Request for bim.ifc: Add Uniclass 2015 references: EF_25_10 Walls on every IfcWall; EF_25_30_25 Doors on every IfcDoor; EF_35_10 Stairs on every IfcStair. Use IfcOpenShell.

First a look at what the model holds.

```python
import ifcopenshell

model = ifcopenshell.open("bim.ifc")
print(model.schema)
print("classifications:", [c.Name for c in model.by_type("IfcClassification")])
for ifc_class in ("IfcDoor", "IfcRoof", "IfcStair", "IfcWall", "IfcWindow"):
    print(ifc_class, len(model.by_type(ifc_class)))
```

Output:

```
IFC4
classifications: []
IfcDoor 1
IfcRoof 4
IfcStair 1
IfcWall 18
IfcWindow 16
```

```python
import ifcopenshell
import ifcopenshell.api.classification

model = ifcopenshell.open("bim.ifc")

system = ifcopenshell.api.classification.add_classification(model, classification="Uniclass 2015")

codes = {
    "IfcWall": ("EF_25_10", "Walls"),
    "IfcDoor": ("EF_25_30_25", "Doors"),
    "IfcStair": ("EF_35_10", "Stairs"),
}
for ifc_class, (code, name) in codes.items():
    products = model.by_type(ifc_class)
    ifcopenshell.api.classification.add_reference(
        model, products=products, classification=system, identification=code, name=name
    )
    print(code, len(products))

model.write("bim_v2.ifc")
```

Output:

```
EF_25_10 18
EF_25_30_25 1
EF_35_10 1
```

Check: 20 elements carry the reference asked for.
